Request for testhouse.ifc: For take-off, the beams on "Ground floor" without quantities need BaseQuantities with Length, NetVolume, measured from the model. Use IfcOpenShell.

First a look at what the model holds.

```python
import ifcopenshell
import ifcopenshell.util.element
import ifcopenshell.util.unit

model = ifcopenshell.open("testhouse.ifc")
print(model.schema)
for unit_type in ("LENGTHUNIT", "AREAUNIT", "VOLUMEUNIT"):
    print(unit_type, ifcopenshell.util.unit.calculate_unit_scale(model, unit_type))
storey = next(s for s in model.by_type("IfcBuildingStorey") if s.Name == "Ground floor")
beams = [e for e in ifcopenshell.util.element.get_decomposition(storey) if e.is_a("IfcBeam")]
for e in sorted(beams, key=lambda e: e.id()):
    print(e.id(), e.is_a(), e.Name, list(ifcopenshell.util.element.get_psets(e, qtos_only=True)), sep=" | ")
```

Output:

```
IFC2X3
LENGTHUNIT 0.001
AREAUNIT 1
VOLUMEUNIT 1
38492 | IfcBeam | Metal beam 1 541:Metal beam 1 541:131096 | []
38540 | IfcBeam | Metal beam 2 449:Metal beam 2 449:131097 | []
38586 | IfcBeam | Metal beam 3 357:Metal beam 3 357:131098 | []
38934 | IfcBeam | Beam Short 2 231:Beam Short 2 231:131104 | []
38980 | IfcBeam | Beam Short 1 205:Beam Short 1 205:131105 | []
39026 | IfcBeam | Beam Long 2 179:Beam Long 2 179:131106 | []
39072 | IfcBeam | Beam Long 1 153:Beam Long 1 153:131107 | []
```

```python
import ifcopenshell
import ifcopenshell.api.pset
import ifcopenshell.geom
import ifcopenshell.util.element
import ifcopenshell.util.shape
import ifcopenshell.util.unit

model = ifcopenshell.open("testhouse.ifc")
unit_scale = ifcopenshell.util.unit.calculate_unit_scale(model)
volume_scale = ifcopenshell.util.unit.calculate_unit_scale(model, "VOLUMEUNIT")
settings = ifcopenshell.geom.settings()

storey = next(s for s in model.by_type("IfcBuildingStorey") if s.Name == "Ground floor")
beams = [e for e in ifcopenshell.util.element.get_decomposition(storey) if e.is_a("IfcBeam")]

for e in sorted(beams, key=lambda e: e.id()):
    if ifcopenshell.util.element.get_psets(e, qtos_only=True, should_inherit=False):
        continue
    # Geometry comes back in metres, in the element's own axes.
    shape = ifcopenshell.geom.create_shape(settings, e)
    values = {
        "Length": ifcopenshell.util.shape.get_max_xyz(shape.geometry) / unit_scale,
        "NetVolume": ifcopenshell.util.shape.get_volume(shape.geometry) / volume_scale,
    }
    qto = ifcopenshell.api.pset.add_qto(model, product=e, name="BaseQuantities")
    ifcopenshell.api.pset.edit_qto(model, qto=qto, properties=values)
    print(e.id(), {k: round(v, 3) for k, v in values.items()})

model.write("testhouse_v2.ifc")
```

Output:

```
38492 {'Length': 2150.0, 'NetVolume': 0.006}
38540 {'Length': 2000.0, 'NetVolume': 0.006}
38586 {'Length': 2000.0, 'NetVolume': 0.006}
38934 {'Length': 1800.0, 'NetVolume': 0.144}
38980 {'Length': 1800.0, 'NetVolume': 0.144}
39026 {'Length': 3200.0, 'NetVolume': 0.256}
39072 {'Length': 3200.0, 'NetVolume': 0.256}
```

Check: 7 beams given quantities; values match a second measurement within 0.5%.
